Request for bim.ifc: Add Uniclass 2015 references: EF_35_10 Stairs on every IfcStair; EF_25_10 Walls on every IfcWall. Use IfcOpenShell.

First a look at what the model holds.

```python
import ifcopenshell

model = ifcopenshell.open("bim.ifc")
print(model.schema)
print("classifications:", [c.Name for c in model.by_type("IfcClassification")])
for ifc_class in ("IfcDoor", "IfcRoof", "IfcStair", "IfcWall", "IfcWindow"):
    print(ifc_class, len(model.by_type(ifc_class)))
```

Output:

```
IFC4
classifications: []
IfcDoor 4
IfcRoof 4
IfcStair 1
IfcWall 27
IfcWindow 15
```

```python
import ifcopenshell
import ifcopenshell.api.classification

model = ifcopenshell.open("bim.ifc")

system = ifcopenshell.api.classification.add_classification(model, classification="Uniclass 2015")

codes = {
    "IfcStair": ("EF_35_10", "Stairs"),
    "IfcWall": ("EF_25_10", "Walls"),
}
for ifc_class, (code, name) in codes.items():
    products = model.by_type(ifc_class)
    ifcopenshell.api.classification.add_reference(
        model, products=products, classification=system, identification=code, name=name
    )
    print(code, len(products))

model.write("bim_edited.ifc")
```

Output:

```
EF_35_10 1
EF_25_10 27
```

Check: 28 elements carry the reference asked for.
